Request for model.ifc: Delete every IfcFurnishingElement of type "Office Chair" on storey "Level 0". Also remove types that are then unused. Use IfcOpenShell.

First a look at what the model holds.

```python
import ifcopenshell
import ifcopenshell.util.element

model = ifcopenshell.open("model.ifc")
print(model.schema)
storey = next(s for s in model.by_type("IfcBuildingStorey") if s.Name == "Level 0")
furniture = [e for e in ifcopenshell.util.element.get_decomposition(storey) if e.is_a("IfcFurnishingElement")]
seen = {}
for e in furniture:
    element_type = ifcopenshell.util.element.get_type(e)
    name = element_type.Name if element_type not in (None, e) else None
    seen[name] = seen.get(name, 0) + 1
for name, count in sorted(seen.items(), key=str):
    print(count, "x", name)
```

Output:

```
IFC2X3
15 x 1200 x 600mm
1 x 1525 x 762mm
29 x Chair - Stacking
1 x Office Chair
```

```python
import ifcopenshell
import ifcopenshell.api.root
import ifcopenshell.util.element

model = ifcopenshell.open("model.ifc")

storey = next(s for s in model.by_type("IfcBuildingStorey") if s.Name == "Level 0")
furniture = [e for e in ifcopenshell.util.element.get_decomposition(storey) if e.is_a("IfcFurnishingElement")]
targets = [e for e in furniture if (t := ifcopenshell.util.element.get_type(e)) not in (None, e) and t.Name == "Office Chair"]
types = {ifcopenshell.util.element.get_type(e) for e in targets} - {None, *targets}

for e in targets:
    ifcopenshell.api.root.remove_product(model, product=e)
print(len(targets), "removed")

unused = [t for t in types if not ifcopenshell.util.element.get_types(t)]
for t in unused:
    ifcopenshell.api.root.remove_product(model, product=t)
print(len(unused), "unused types removed")

model.write("model_edited.ifc")
```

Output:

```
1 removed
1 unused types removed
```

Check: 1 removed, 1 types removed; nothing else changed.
